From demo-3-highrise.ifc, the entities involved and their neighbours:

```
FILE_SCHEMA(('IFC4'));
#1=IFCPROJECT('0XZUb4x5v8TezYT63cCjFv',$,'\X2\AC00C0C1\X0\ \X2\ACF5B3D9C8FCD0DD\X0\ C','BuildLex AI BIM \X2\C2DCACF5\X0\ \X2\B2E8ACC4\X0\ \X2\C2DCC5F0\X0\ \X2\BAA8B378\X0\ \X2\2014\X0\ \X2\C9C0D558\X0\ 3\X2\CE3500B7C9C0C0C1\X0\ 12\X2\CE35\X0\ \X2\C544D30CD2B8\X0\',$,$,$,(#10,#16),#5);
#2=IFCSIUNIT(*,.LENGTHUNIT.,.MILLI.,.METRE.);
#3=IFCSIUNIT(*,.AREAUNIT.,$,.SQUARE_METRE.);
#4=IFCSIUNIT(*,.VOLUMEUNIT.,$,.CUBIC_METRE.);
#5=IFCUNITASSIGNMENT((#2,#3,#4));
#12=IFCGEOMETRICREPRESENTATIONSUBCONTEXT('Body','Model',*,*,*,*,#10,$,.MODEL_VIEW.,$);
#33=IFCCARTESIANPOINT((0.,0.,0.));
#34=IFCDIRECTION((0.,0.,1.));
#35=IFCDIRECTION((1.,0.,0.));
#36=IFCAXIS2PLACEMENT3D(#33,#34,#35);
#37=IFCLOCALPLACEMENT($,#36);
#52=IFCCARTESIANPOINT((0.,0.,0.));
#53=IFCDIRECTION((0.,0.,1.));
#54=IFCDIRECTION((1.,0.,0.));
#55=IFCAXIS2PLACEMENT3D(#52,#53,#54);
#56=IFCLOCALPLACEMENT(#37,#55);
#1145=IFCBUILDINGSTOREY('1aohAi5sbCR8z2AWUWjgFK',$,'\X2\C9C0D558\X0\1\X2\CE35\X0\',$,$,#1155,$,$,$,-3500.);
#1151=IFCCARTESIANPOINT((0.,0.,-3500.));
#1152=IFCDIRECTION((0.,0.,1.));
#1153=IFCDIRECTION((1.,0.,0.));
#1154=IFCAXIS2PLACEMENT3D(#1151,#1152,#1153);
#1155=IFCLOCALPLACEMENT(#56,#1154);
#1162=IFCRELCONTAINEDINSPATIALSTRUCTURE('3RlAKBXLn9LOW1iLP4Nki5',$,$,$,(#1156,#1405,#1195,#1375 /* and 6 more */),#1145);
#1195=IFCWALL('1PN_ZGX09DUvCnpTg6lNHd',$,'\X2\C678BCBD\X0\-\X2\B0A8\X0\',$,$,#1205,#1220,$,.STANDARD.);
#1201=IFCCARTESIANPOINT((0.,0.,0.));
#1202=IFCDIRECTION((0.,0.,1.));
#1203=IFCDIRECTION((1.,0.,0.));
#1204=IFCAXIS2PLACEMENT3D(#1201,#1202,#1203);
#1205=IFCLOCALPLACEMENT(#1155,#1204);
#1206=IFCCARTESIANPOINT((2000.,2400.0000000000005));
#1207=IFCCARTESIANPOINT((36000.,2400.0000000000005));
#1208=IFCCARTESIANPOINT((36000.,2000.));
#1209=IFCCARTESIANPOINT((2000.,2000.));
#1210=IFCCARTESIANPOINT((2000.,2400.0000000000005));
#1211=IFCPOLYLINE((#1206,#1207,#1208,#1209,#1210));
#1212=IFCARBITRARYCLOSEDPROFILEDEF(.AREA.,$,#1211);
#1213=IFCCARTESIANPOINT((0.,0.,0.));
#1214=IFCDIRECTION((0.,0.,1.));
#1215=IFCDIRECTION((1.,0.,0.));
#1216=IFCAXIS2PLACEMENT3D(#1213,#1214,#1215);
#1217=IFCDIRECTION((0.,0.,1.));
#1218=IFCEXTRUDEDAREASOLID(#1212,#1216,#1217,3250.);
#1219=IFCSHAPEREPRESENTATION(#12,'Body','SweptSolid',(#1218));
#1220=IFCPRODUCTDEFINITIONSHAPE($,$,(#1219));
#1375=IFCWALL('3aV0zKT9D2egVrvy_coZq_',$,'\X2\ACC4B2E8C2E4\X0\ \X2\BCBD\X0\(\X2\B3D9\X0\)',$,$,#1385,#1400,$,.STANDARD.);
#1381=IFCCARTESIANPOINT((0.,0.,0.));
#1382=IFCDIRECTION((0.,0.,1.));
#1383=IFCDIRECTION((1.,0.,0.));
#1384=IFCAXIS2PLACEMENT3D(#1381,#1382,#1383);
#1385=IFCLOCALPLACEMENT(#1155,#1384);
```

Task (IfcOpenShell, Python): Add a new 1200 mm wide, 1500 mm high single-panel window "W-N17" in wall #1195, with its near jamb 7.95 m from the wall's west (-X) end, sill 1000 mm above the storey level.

```python
import numpy as np
import ifcopenshell
import ifcopenshell.api.feature
import ifcopenshell.api.geometry
import ifcopenshell.api.root
import ifcopenshell.api.spatial
import ifcopenshell.geom
import ifcopenshell.util.element
import ifcopenshell.util.placement
import ifcopenshell.util.representation
import ifcopenshell.util.shape
import ifcopenshell.util.unit

model = ifcopenshell.open("demo-3-highrise.ifc")
unit_scale = ifcopenshell.util.unit.calculate_unit_scale(model)
settings = ifcopenshell.geom.settings()


def volume(element):
    """Net volume in cubic metres, openings subtracted."""
    shape = ifcopenshell.geom.create_shape(settings, element)
    return ifcopenshell.util.shape.get_volume(shape.geometry)


wall = model.by_guid("1PN_ZGX09DUvCnpTg6lNHd")
storey = ifcopenshell.util.element.get_container(wall, ifc_class="IfcBuildingStorey")
context = ifcopenshell.util.representation.get_context(model, "Model", "Body", "MODEL_VIEW")
before = volume(wall)

width, height, from_end, sill = 1.2, 1.5, 7.95, 1  # metres

# The wall runs along its own X axis, and the end named is its -X end.
wall_shape = ifcopenshell.geom.create_shape(settings, wall)
x, y, z = ifcopenshell.util.shape.get_vertices(wall_shape.geometry).T
start = x.min() + from_end
face, thickness = float(y.min()), float(y.max() - y.min())
wall_matrix = ifcopenshell.util.placement.get_local_placement(wall.ObjectPlacement)
level = ifcopenshell.util.placement.get_local_placement(storey.ObjectPlacement)[2, 3]


def in_wall(x, y):
    """Placement at x, y metres in the wall's axes, at sill height."""
    matrix = wall_matrix.copy()
    matrix[:, 3] = wall_matrix @ np.array([x / unit_scale, y / unit_scale, 0.0, 1.0])
    matrix[2, 3] = level + sill / unit_scale
    return matrix


# Opening: a box that overshoots both wall faces by 50 mm.
opening = ifcopenshell.api.root.create_entity(model, ifc_class="IfcOpeningElement", predefined_type="OPENING")
box = ifcopenshell.api.geometry.add_wall_representation(
    model, context=context, length=width, height=height, thickness=thickness + 0.1
)
ifcopenshell.api.geometry.assign_representation(model, product=opening, representation=box)
ifcopenshell.api.geometry.edit_object_placement(model, product=opening, matrix=in_wall(start, face - 0.05), is_si=False)
ifcopenshell.api.feature.add_feature(model, feature=opening, element=wall)

window = ifcopenshell.api.root.create_entity(model, ifc_class="IfcWindow", name="W-N17", predefined_type="WINDOW")
window.OverallWidth, window.OverallHeight = width / unit_scale, height / unit_scale
window.PartitioningType = "SINGLE_PANEL"
body = ifcopenshell.api.geometry.add_window_representation(
    model,
    context=context,
    overall_width=window.OverallWidth,
    overall_height=window.OverallHeight,
    partition_type="SINGLE_PANEL",
)
ifcopenshell.api.geometry.assign_representation(model, product=window, representation=body)
ifcopenshell.api.spatial.assign_container(model, products=[window], relating_structure=storey)
ifcopenshell.api.feature.add_filling(model, opening=opening, element=window)

# Centre the window in the wall's thickness.
ifcopenshell.api.geometry.edit_object_placement(model, product=window, matrix=in_wall(start, face), is_si=False)
window_shape = ifcopenshell.geom.create_shape(settings, window)
depth = ifcopenshell.util.shape.get_vertices(window_shape.geometry)[:, 1]
offset = face + thickness / 2 - (depth.min() + depth.max()) / 2
ifcopenshell.api.geometry.edit_object_placement(model, product=window, matrix=in_wall(start, offset), is_si=False)

after = volume(wall)

print(f"wall volume {before:.3f} -> {after:.3f} m3")

model.write("demo-3-highrise_v2.ifc")
```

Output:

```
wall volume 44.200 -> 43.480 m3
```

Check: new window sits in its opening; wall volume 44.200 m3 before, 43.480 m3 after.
